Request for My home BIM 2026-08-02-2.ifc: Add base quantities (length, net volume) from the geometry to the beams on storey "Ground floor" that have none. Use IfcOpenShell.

First a look at what the model holds.

```python
import ifcopenshell
import ifcopenshell.util.element
import ifcopenshell.util.unit

model = ifcopenshell.open("My home BIM 2026-08-02-2.ifc")
print(model.schema)
for unit_type in ("LENGTHUNIT", "AREAUNIT", "VOLUMEUNIT"):
    print(unit_type, ifcopenshell.util.unit.calculate_unit_scale(model, unit_type))
storey = next(s for s in model.by_type("IfcBuildingStorey") if s.Name == "Ground floor")
beams = [e for e in ifcopenshell.util.element.get_decomposition(storey) if e.is_a("IfcBeam")]
for e in sorted(beams, key=lambda e: e.id()):
    print(e.id(), e.is_a(), e.Name, list(ifcopenshell.util.element.get_psets(e, qtos_only=True)), sep=" | ")
```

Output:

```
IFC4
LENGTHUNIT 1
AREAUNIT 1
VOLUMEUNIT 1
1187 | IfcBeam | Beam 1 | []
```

```python
import ifcopenshell
import ifcopenshell.api.pset
import ifcopenshell.geom
import ifcopenshell.util.element
import ifcopenshell.util.shape
import ifcopenshell.util.unit

model = ifcopenshell.open("My home BIM 2026-08-02-2.ifc")
unit_scale = ifcopenshell.util.unit.calculate_unit_scale(model)
volume_scale = ifcopenshell.util.unit.calculate_unit_scale(model, "VOLUMEUNIT")
settings = ifcopenshell.geom.settings()

storey = next(s for s in model.by_type("IfcBuildingStorey") if s.Name == "Ground floor")
beams = [e for e in ifcopenshell.util.element.get_decomposition(storey) if e.is_a("IfcBeam")]

for e in sorted(beams, key=lambda e: e.id()):
    if ifcopenshell.util.element.get_psets(e, qtos_only=True, should_inherit=False):
        continue
    # Geometry comes back in metres, in the element's own axes.
    shape = ifcopenshell.geom.create_shape(settings, e)
    values = {
        "Length": ifcopenshell.util.shape.get_max_xyz(shape.geometry) / unit_scale,
        "NetVolume": ifcopenshell.util.shape.get_volume(shape.geometry) / volume_scale,
    }
    qto = ifcopenshell.api.pset.add_qto(model, product=e, name="Qto_BeamBaseQuantities")
    ifcopenshell.api.pset.edit_qto(model, qto=qto, properties=values)
    print(e.id(), {k: round(v, 3) for k, v in values.items()})

model.write("My home BIM 2026-08-02-2_rev.ifc")
```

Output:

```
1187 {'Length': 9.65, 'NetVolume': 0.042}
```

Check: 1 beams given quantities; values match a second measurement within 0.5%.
